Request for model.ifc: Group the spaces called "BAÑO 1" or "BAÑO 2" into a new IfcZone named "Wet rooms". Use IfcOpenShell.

First a look at what the model holds.

```python
import ifcopenshell

model = ifcopenshell.open("model.ifc")
print(model.schema)
seen = {}
for space in model.by_type("IfcSpace"):
    seen[space.LongName] = seen.get(space.LongName, 0) + 1
for name, count in sorted(seen.items(), key=str):
    print(count, "x", name)
print("zones:", [z.Name for z in model.by_type("IfcZone")][:20])
```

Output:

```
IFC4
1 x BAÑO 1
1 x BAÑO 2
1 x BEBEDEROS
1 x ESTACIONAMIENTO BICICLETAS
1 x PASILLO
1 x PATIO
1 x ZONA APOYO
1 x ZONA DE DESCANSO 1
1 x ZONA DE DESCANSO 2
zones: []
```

```python
import ifcopenshell
import ifcopenshell.api.group
import ifcopenshell.api.root

model = ifcopenshell.open("model.ifc")

names = {"BAÑO 1", "BAÑO 2"}
spaces = [s for s in model.by_type("IfcSpace") if s.LongName in names]

zone = ifcopenshell.api.root.create_entity(model, ifc_class="IfcZone", name="Wet rooms")
ifcopenshell.api.group.assign_group(model, products=spaces, group=zone)
print(len(spaces), "spaces in", zone.Name)

model.write("model_v2.ifc")
```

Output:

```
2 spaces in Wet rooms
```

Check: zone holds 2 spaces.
